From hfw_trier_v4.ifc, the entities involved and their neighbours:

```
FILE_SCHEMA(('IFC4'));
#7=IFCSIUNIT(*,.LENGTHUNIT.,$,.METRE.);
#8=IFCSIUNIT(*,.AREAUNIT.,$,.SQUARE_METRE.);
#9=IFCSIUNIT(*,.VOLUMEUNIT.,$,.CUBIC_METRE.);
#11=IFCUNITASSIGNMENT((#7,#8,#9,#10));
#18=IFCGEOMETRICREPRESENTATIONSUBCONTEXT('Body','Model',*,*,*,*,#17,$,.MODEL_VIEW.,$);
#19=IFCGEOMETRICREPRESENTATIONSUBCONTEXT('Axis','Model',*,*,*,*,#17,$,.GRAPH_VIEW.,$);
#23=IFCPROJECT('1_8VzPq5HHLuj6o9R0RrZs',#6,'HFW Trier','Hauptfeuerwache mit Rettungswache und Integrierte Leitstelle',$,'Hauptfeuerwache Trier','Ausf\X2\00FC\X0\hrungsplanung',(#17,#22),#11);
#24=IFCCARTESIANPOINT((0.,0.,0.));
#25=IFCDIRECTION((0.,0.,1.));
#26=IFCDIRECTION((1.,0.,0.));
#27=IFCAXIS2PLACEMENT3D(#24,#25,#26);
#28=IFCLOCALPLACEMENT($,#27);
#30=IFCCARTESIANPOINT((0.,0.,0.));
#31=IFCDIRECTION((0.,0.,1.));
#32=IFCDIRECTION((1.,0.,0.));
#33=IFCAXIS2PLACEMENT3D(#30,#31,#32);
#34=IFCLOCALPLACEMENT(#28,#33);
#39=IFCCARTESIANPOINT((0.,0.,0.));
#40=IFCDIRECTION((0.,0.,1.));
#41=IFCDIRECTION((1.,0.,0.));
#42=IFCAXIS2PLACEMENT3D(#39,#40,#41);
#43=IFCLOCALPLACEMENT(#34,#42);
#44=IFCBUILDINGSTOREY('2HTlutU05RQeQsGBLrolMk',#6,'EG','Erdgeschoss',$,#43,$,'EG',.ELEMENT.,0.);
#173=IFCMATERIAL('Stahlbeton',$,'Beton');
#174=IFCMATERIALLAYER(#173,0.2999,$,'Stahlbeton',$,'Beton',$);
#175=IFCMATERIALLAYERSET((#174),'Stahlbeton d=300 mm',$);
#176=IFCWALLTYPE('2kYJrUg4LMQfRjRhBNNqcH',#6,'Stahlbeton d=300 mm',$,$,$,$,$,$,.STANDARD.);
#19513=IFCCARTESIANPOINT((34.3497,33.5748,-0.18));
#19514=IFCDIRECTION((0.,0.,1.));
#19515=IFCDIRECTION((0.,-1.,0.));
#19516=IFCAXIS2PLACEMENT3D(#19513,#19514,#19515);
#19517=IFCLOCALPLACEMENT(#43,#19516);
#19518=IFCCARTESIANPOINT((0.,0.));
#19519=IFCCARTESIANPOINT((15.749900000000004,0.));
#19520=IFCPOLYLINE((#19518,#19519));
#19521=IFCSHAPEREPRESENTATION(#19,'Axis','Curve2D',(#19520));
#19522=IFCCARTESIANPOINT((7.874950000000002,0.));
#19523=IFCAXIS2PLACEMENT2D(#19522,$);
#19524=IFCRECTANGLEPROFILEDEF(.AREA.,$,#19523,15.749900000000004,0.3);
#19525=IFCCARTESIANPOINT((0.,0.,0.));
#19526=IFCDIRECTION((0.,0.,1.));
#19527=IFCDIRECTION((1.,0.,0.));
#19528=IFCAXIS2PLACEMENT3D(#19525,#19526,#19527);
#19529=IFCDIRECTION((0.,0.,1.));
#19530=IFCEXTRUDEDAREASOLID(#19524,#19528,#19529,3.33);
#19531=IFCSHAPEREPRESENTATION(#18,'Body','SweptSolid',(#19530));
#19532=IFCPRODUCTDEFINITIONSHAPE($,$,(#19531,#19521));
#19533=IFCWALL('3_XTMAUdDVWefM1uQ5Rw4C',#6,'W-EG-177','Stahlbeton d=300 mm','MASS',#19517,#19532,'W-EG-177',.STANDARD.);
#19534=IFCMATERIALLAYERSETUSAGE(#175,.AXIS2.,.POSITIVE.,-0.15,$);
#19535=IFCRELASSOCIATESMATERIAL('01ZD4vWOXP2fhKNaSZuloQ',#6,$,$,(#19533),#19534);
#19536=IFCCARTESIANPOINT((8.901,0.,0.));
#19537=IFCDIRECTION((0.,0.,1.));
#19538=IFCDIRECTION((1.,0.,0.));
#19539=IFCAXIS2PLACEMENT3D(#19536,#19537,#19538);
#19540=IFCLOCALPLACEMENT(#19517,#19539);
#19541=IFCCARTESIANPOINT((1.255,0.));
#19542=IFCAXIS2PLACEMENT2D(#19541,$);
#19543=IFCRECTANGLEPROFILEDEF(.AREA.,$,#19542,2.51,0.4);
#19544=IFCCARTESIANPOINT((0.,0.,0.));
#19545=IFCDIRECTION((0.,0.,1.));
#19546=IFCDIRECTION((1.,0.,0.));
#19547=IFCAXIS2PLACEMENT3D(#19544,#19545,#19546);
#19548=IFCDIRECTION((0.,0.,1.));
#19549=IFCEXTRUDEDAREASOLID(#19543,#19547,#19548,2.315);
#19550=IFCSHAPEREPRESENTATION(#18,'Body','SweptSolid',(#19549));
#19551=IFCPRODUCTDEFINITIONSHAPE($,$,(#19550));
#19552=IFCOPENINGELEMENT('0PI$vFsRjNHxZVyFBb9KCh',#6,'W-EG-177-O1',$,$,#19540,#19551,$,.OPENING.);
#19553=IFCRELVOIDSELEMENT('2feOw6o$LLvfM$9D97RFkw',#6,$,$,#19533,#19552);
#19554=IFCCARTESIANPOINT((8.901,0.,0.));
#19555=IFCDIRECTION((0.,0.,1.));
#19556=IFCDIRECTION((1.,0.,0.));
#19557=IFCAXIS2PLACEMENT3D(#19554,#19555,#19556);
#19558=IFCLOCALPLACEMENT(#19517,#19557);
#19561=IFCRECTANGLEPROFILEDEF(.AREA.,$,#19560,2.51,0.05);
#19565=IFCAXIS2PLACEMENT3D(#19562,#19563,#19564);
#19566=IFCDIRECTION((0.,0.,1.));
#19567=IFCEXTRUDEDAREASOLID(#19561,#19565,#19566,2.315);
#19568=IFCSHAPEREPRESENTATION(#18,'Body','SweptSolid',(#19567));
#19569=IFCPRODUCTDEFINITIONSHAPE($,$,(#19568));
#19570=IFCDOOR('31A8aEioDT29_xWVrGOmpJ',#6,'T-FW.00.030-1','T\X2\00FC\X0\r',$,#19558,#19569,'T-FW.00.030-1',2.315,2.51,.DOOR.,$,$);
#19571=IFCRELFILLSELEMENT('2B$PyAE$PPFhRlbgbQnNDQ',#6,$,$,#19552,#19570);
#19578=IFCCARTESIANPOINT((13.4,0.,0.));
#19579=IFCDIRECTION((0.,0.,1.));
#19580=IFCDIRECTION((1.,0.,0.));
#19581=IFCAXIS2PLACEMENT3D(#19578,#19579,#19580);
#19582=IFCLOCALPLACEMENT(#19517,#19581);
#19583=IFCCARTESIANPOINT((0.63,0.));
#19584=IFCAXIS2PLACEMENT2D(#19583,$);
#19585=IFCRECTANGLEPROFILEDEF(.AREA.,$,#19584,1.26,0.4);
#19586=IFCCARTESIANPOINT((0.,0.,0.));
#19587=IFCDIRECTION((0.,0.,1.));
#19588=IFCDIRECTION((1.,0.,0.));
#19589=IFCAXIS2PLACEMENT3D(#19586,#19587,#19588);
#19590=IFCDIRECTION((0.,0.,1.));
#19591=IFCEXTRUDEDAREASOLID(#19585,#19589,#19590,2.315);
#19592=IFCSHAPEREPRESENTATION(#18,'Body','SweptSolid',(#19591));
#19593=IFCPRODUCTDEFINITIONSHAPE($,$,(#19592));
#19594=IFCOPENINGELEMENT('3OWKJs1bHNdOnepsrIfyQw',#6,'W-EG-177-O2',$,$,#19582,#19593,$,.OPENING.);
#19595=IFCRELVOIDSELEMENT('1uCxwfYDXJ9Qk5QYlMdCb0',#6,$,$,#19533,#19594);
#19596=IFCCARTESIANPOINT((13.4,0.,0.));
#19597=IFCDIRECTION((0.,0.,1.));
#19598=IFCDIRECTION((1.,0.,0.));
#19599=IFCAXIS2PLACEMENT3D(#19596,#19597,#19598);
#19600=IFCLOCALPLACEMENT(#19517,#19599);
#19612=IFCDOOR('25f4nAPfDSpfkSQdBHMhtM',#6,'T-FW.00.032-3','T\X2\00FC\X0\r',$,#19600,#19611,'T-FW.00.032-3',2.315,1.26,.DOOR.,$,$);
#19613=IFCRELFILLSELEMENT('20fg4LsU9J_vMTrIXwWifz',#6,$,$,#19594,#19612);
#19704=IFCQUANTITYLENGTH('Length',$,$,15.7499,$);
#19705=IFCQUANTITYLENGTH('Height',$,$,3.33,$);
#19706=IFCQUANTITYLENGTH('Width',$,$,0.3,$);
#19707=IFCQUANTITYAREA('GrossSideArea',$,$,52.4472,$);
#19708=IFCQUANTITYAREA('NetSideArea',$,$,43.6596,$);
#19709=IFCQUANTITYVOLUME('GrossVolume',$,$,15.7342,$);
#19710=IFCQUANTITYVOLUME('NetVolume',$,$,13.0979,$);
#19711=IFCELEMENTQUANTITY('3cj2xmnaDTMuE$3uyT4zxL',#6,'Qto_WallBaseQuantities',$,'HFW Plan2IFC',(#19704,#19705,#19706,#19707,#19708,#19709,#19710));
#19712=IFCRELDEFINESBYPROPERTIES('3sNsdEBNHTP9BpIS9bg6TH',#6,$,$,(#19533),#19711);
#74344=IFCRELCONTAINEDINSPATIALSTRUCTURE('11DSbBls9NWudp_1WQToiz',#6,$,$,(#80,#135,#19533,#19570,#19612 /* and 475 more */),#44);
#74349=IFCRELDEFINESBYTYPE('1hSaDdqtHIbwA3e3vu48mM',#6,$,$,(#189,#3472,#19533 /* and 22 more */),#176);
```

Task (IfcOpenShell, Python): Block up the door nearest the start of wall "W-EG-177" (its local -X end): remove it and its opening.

```python
import ifcopenshell
import ifcopenshell.api.feature
import ifcopenshell.api.pset
import ifcopenshell.api.root
import ifcopenshell.geom
import ifcopenshell.util.element
import ifcopenshell.util.shape
import ifcopenshell.util.unit

model = ifcopenshell.open("hfw_trier_v4.ifc")
area_scale = ifcopenshell.util.unit.calculate_unit_scale(model, "AREAUNIT")
volume_scale = ifcopenshell.util.unit.calculate_unit_scale(model, "VOLUMEUNIT")
settings = ifcopenshell.geom.settings()


def volume(element):
    """Net volume in cubic metres, openings subtracted."""
    shape = ifcopenshell.geom.create_shape(settings, element)
    return ifcopenshell.util.shape.get_volume(shape.geometry)


door = model.by_id(19570)
opening = door.FillsVoids[0].RelatingOpeningElement
wall = opening.VoidsElements[0].RelatingBuildingElement
before = volume(wall)

ifcopenshell.api.root.remove_product(model, product=door)
ifcopenshell.api.feature.remove_feature(model, feature=opening)

after = volume(wall)
thickness = 0.3  # wall thickness in metres

# Update the wall's stored quantities.
qto = model.by_id(ifcopenshell.util.element.get_pset(wall, "Qto_WallBaseQuantities", should_inherit=False)["id"])
ifcopenshell.api.pset.edit_qto(model, qto=qto, properties={
    "NetSideArea": after / thickness / area_scale,
    "NetVolume": after / volume_scale,
})

print(f"wall volume {before:.3f} -> {after:.3f} m3")

model.write("hfw_trier_v4_v2.ifc")
```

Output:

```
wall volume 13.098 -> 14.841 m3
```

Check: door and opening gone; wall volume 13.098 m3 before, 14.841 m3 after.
